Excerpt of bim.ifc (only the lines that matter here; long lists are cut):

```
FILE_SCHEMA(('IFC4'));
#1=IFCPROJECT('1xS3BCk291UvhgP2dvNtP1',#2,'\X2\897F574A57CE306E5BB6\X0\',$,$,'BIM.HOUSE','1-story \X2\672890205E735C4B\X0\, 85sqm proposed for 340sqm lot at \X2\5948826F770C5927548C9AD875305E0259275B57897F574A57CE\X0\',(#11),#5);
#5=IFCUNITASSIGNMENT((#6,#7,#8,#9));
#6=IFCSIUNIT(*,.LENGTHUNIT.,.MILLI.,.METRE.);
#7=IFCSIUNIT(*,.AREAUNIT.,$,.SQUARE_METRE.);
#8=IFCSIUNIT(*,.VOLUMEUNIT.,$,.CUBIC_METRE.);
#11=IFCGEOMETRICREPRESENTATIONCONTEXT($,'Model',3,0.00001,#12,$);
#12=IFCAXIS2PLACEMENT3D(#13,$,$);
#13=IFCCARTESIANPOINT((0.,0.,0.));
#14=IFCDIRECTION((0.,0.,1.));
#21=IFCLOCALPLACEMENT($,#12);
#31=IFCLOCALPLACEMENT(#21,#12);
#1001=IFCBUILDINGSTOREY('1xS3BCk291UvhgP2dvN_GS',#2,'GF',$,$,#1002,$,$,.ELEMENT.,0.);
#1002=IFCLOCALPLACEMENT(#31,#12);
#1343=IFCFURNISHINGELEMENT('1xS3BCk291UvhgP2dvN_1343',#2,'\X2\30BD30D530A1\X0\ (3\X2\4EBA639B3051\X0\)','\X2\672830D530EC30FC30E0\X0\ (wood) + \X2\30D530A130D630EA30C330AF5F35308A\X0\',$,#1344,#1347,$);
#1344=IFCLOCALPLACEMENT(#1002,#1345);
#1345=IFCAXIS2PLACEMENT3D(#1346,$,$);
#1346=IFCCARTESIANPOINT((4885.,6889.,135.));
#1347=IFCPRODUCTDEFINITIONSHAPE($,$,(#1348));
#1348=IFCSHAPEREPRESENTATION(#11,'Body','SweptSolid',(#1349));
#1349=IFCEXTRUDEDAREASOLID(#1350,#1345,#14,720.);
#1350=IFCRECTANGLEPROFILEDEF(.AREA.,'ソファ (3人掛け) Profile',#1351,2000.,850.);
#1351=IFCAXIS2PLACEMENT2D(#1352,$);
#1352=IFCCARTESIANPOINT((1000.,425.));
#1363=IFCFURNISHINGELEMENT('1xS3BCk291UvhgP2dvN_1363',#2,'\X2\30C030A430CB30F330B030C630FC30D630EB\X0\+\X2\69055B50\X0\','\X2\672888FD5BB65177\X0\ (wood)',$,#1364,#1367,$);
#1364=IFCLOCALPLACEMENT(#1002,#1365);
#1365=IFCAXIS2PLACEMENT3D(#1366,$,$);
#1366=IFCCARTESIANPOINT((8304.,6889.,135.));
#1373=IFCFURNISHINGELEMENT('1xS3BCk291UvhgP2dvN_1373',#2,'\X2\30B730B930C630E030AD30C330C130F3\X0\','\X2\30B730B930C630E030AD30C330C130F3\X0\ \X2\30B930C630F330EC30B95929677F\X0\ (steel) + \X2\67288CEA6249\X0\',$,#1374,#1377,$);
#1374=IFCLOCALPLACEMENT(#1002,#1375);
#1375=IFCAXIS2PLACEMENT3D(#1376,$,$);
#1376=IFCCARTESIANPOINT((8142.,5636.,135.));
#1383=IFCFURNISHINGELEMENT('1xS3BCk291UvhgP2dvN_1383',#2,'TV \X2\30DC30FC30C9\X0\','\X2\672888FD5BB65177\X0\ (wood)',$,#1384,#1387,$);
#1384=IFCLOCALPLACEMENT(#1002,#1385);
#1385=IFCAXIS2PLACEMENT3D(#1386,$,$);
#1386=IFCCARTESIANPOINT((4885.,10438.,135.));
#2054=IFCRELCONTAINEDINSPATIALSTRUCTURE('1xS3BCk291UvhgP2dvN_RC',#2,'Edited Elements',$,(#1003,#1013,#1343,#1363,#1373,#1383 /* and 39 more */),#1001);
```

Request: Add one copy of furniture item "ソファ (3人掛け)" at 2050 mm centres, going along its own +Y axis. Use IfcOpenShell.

```python
import ifcopenshell
import ifcopenshell.api.geometry
import ifcopenshell.api.root
import ifcopenshell.util.element
import ifcopenshell.util.placement
import ifcopenshell.util.unit

model = ifcopenshell.open("bim.ifc")
unit_scale = ifcopenshell.util.unit.calculate_unit_scale(model)


def reuse_history(source, copy):
    """copy_class also copies each property set's owner history, people and application; keep the originals."""
    for rel in copy.IsDefinedBy:
        if rel.is_a("IfcRelDefinesByProperties") and (history := rel.RelatingPropertyDefinition.OwnerHistory):
            rel.RelatingPropertyDefinition.OwnerHistory = source.OwnerHistory
            ifcopenshell.util.element.remove_deep2(model, history)


source = model.by_guid("1xS3BCk291UvhgP2dvN_1343")
base = ifcopenshell.util.placement.get_local_placement(source.ObjectPlacement)
step = base[:3, 1] * 2.05 / unit_scale

for i in range(1, 2):
    copy = ifcopenshell.api.root.copy_class(model, product=source)
    copy.Representation = ifcopenshell.util.element.copy_deep(
        model, source.Representation, exclude=["IfcGeometricRepresentationContext", "IfcRepresentationMap"]
    )
    reuse_history(source, copy)
    matrix = base.copy()
    matrix[:3, 3] += i * step
    print("added at", matrix[:3, 3].round(3) + 0.0)
    ifcopenshell.api.geometry.edit_object_placement(model, product=copy, matrix=matrix, is_si=False)

model.write("bim_rev.ifc")
```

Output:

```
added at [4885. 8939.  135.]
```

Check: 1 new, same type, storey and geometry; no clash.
